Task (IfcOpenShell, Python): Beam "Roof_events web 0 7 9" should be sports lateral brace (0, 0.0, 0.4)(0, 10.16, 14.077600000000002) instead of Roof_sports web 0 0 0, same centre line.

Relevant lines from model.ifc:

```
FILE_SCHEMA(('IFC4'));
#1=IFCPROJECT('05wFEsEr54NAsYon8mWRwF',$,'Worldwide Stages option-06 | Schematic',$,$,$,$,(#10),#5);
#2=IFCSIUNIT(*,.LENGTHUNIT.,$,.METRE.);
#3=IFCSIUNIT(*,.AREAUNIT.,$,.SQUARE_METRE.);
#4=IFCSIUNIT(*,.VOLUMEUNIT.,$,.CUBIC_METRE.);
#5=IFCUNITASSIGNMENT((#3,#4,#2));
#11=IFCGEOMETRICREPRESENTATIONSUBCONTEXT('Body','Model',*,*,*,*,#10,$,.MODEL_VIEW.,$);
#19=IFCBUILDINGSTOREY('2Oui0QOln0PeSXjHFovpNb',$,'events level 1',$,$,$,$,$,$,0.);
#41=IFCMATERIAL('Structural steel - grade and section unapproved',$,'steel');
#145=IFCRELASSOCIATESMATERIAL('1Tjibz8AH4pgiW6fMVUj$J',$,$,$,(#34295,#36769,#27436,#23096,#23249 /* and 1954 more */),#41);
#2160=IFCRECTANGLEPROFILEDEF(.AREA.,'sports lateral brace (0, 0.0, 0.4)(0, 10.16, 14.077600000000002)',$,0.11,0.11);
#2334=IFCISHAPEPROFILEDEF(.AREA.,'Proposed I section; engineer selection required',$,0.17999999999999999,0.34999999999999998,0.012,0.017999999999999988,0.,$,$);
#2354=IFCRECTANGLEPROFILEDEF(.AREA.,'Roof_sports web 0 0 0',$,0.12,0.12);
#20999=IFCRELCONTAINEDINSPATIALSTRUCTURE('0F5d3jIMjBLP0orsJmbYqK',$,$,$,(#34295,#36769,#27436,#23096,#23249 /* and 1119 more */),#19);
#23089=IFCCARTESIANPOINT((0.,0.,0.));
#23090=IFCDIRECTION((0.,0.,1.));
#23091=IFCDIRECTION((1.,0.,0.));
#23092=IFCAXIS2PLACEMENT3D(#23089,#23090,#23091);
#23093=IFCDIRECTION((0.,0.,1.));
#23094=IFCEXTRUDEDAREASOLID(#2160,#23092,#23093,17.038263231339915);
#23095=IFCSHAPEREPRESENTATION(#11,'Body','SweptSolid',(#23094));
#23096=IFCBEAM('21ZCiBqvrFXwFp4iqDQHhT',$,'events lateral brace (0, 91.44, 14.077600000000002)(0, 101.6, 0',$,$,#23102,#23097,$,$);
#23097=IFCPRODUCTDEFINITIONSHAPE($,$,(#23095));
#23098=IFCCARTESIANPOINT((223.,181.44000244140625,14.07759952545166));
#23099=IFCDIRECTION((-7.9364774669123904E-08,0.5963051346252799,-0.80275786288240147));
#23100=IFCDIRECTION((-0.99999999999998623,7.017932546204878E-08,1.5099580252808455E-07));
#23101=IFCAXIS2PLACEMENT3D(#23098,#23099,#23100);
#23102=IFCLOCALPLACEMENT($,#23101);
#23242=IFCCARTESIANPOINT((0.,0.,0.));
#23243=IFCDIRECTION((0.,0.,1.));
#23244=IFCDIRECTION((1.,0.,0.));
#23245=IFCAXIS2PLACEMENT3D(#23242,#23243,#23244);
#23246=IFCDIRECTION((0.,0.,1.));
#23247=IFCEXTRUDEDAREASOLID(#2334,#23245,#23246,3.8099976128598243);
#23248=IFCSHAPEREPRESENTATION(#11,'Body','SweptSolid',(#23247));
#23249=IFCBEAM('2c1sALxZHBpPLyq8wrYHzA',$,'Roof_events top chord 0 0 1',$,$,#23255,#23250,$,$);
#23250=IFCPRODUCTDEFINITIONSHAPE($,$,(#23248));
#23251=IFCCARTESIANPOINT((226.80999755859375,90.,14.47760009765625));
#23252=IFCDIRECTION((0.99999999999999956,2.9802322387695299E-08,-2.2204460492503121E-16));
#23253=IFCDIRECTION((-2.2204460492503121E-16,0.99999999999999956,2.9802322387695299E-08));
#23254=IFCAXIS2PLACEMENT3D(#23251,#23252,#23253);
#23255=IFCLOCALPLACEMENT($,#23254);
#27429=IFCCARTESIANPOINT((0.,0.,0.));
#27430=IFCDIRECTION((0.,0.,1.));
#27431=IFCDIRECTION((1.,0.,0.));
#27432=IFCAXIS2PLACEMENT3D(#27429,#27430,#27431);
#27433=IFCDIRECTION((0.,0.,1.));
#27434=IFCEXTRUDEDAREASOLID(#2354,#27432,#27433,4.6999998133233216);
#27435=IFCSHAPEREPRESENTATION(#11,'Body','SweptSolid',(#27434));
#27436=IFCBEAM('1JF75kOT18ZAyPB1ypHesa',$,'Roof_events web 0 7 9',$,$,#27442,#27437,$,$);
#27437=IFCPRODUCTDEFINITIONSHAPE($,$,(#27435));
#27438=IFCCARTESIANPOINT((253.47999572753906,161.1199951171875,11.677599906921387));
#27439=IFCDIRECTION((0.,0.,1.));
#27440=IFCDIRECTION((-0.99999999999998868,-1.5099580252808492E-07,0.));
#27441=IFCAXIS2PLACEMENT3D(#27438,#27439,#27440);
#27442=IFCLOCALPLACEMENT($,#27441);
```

```python
import ifcopenshell
import ifcopenshell.util.element
import ifcopenshell.util.representation

model = ifcopenshell.open("model.ifc")

member = model.by_guid("1JF75kOT18ZAyPB1ypHesa")
source = next(p for p in model.by_type("IfcRectangleProfileDef") if p.ProfileName == "sports lateral brace (0, 0.0, 0.4)(0, 10.16, 14.077600000000002)")

body = ifcopenshell.util.representation.get_representation(member, "Model", "Body")
solid = body.Items[0]
old_profile = solid.SweptArea

# Copy the section's sizes but keep this member's own profile position.
profile = ifcopenshell.util.element.copy(model, source)
profile.Position = old_profile.Position
solid.SweptArea = profile
if not model.get_total_inverses(old_profile):
    ifcopenshell.util.element.remove_deep2(model, old_profile)

print(solid.SweptArea)

model.write("model_updated.ifc")
```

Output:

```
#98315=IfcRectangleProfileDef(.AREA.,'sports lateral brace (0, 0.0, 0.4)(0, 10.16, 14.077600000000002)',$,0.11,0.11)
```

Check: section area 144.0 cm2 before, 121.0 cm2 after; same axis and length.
